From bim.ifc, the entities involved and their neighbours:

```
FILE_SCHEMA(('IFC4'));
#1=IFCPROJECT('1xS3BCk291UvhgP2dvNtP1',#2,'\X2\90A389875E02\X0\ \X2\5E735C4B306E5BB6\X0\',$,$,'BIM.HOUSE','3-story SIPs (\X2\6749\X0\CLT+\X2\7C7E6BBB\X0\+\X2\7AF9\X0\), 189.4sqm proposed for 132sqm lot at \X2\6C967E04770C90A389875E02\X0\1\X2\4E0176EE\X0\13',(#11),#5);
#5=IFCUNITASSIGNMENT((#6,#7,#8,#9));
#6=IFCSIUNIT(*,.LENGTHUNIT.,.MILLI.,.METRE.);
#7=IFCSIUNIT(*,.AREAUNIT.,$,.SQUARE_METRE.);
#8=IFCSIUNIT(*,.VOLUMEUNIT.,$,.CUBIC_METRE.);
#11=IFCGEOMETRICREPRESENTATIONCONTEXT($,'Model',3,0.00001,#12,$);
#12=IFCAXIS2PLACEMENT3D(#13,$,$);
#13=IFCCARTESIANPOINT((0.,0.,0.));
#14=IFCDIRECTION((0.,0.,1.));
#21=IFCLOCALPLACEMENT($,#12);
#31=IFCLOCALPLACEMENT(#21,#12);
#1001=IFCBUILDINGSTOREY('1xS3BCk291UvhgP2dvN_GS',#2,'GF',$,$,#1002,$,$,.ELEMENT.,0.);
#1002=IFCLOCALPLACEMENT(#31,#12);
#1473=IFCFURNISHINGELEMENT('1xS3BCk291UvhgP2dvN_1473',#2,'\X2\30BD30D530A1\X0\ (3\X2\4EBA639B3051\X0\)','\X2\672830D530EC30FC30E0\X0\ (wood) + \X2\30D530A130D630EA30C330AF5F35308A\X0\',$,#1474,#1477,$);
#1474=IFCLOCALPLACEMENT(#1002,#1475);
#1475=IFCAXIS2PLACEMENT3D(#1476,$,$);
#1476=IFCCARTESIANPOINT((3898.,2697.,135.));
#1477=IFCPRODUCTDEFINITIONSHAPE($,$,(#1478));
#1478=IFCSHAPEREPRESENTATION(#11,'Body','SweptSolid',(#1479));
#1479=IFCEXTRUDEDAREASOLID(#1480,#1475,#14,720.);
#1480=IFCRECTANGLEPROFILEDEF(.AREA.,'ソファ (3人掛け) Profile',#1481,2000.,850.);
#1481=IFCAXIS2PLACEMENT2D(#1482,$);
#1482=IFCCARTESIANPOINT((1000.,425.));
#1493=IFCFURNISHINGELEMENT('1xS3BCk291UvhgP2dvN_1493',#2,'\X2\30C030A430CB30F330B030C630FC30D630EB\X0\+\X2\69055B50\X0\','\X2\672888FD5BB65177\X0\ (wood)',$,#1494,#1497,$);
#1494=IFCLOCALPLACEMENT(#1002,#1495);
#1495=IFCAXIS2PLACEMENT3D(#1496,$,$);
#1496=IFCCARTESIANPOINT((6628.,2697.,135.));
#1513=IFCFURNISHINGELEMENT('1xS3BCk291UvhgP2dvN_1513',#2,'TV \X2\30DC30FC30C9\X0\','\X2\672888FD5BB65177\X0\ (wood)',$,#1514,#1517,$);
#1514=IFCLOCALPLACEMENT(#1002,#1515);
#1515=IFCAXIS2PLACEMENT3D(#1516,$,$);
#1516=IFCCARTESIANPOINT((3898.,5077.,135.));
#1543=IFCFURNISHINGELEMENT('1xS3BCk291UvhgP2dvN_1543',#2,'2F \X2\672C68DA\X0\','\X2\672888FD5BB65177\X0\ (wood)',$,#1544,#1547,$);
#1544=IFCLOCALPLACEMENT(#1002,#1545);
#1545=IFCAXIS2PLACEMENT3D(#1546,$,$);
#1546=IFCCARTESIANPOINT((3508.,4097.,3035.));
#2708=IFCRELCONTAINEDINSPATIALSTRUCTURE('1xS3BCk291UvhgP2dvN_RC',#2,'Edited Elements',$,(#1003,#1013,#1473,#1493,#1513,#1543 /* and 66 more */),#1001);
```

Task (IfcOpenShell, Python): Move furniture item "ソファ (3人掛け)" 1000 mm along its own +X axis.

```python
import ifcopenshell
import ifcopenshell.api.geometry
import ifcopenshell.util.placement
import ifcopenshell.util.unit

model = ifcopenshell.open("bim.ifc")
unit_scale = ifcopenshell.util.unit.calculate_unit_scale(model)

item = model.by_guid("1xS3BCk291UvhgP2dvN_1473")
matrix = ifcopenshell.util.placement.get_local_placement(item.ObjectPlacement)
matrix[:3, 3] += matrix[:3, 0] * 1 / unit_scale
ifcopenshell.api.geometry.edit_object_placement(model, product=item, matrix=matrix, is_si=False)

print(ifcopenshell.util.placement.get_local_placement(item.ObjectPlacement).round(3) + 0.0)

model.write("bim_updated.ifc")
```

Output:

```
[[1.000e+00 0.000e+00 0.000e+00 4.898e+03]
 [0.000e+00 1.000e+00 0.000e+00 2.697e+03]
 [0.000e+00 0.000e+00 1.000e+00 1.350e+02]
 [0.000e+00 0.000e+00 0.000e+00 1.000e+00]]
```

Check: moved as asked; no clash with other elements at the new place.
